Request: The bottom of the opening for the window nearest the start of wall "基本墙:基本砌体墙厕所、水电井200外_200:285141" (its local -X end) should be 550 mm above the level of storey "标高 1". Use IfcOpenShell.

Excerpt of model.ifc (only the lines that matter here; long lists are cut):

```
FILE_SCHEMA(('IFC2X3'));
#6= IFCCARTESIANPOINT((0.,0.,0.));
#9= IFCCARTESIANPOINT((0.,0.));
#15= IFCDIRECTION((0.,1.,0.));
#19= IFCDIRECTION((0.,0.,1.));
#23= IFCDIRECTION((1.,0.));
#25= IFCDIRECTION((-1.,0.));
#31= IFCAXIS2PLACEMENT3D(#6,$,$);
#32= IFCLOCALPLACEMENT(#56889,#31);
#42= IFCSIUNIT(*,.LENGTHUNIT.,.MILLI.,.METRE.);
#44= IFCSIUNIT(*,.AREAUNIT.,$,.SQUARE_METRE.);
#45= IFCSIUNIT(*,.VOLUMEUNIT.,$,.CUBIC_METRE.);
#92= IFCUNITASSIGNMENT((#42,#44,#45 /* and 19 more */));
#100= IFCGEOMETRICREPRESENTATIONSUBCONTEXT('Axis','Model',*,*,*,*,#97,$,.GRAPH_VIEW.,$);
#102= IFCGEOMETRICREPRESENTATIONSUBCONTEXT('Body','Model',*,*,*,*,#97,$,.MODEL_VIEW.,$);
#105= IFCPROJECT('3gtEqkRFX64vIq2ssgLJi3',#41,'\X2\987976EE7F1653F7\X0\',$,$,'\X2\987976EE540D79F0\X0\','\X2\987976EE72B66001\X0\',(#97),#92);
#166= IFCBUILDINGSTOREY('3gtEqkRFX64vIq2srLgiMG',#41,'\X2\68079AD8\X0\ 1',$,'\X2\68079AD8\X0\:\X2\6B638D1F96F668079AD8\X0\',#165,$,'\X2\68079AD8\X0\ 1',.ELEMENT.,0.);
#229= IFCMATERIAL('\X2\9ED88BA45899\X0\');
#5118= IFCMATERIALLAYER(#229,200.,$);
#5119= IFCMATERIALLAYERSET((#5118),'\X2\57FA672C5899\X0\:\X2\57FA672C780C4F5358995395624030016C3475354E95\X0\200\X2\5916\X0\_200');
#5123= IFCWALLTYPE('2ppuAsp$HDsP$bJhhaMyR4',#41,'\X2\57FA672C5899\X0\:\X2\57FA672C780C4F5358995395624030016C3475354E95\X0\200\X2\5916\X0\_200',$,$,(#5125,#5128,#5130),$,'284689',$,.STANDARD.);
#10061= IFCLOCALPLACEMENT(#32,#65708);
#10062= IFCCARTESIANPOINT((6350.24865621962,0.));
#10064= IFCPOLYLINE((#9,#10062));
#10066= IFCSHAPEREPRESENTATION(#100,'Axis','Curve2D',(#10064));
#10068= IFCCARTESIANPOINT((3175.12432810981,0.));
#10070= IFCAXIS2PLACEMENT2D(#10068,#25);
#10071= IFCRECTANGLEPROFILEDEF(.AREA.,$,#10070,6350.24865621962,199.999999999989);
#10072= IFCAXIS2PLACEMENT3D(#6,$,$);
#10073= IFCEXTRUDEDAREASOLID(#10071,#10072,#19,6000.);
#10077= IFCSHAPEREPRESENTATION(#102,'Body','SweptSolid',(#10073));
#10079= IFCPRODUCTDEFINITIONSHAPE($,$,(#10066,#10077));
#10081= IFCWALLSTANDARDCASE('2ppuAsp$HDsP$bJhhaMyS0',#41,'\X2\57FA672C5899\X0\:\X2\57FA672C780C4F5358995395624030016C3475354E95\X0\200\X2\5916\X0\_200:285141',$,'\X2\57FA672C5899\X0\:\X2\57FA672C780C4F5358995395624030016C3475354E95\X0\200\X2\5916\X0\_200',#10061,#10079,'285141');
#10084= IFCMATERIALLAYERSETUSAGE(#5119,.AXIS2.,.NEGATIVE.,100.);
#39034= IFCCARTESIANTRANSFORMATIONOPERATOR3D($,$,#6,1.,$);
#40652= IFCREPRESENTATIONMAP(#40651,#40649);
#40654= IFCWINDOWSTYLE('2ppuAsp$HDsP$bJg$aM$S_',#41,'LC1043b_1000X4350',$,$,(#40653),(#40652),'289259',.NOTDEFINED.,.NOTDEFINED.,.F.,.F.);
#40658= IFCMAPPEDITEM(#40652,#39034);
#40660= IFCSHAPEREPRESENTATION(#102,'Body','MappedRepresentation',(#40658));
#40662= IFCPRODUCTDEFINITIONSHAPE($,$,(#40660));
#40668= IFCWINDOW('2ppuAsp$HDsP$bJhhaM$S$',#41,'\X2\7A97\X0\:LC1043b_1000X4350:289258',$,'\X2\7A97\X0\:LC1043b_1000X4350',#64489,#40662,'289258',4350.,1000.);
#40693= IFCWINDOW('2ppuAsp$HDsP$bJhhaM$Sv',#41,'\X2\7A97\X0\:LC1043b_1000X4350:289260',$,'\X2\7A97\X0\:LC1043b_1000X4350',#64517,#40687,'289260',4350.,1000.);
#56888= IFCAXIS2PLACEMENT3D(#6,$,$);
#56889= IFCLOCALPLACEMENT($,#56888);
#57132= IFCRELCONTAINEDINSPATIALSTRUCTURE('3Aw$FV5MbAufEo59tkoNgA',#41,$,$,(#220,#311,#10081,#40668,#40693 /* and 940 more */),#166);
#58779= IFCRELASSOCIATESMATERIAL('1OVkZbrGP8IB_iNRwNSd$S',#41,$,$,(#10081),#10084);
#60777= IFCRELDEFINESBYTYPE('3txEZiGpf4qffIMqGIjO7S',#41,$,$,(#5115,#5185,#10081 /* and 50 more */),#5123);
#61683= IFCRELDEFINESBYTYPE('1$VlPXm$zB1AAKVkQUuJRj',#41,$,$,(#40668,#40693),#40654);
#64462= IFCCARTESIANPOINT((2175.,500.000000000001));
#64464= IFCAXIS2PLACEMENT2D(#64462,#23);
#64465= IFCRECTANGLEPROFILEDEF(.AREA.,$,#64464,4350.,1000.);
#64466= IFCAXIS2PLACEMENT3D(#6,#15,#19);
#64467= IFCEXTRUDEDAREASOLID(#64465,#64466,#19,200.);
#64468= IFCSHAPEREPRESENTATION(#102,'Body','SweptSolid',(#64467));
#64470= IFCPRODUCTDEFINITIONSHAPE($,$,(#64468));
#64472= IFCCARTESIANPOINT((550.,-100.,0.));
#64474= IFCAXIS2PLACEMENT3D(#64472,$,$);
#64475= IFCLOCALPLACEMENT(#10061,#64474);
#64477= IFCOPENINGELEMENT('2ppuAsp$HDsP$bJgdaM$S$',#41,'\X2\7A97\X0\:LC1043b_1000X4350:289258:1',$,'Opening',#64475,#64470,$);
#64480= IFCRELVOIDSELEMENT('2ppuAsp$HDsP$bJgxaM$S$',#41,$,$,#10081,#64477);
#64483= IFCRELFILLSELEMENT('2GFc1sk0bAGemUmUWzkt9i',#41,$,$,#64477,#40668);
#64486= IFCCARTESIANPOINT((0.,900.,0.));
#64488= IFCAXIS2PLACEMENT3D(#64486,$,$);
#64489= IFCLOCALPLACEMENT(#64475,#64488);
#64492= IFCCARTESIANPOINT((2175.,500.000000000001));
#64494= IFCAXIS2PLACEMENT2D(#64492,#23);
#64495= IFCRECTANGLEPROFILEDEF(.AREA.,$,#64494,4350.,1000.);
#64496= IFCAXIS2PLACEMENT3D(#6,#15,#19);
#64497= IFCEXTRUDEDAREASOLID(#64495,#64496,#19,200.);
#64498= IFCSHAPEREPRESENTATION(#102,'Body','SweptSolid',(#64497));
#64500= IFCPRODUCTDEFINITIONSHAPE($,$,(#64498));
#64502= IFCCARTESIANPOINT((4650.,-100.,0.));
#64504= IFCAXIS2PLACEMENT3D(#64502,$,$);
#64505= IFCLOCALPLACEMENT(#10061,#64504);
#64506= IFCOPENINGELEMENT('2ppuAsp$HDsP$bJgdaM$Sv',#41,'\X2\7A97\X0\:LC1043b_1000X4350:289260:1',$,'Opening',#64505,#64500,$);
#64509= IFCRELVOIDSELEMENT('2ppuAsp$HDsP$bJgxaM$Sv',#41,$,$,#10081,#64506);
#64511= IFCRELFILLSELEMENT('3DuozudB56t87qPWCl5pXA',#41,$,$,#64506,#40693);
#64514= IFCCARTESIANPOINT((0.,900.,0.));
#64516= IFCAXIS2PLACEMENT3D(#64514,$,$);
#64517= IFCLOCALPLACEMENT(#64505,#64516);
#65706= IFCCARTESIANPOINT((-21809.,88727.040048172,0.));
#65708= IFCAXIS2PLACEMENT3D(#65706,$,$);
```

```python
import numpy as np
import ifcopenshell
import ifcopenshell.api.geometry
import ifcopenshell.geom
import ifcopenshell.util.element
import ifcopenshell.util.placement
import ifcopenshell.util.shape
import ifcopenshell.util.unit

model = ifcopenshell.open("model.ifc")
unit_scale = ifcopenshell.util.unit.calculate_unit_scale(model)

window = model.by_guid("2ppuAsp$HDsP$bJhhaM$S$")
opening = window.FillsVoids[0].RelatingOpeningElement
storey = ifcopenshell.util.element.get_container(window, ifc_class="IfcBuildingStorey")
level = ifcopenshell.util.placement.get_local_placement(storey.ObjectPlacement)[2, 3]

# The opening's origin need not be at the sill, so measure its lowest point.
shape = ifcopenshell.geom.create_shape(ifcopenshell.geom.settings(), opening)
bottom = ifcopenshell.util.shape.get_shape_bottom_elevation(shape, shape.geometry) / unit_scale
dz = level + 0.55 / unit_scale - bottom

shift = np.array([0.0, 0.0, dz])
# The window is placed relative to its opening, so it follows when the opening moves.
matrix = ifcopenshell.util.placement.get_local_placement(opening.ObjectPlacement)
matrix[:3, 3] += shift
ifcopenshell.api.geometry.edit_object_placement(
    model, product=opening, matrix=matrix, is_si=False, should_transform_children=True
)

print(f"moved by {dz * unit_scale:+.3f} m")

model.write("model_edited.ifc")
```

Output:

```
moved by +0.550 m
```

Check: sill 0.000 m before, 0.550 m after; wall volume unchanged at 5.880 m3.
